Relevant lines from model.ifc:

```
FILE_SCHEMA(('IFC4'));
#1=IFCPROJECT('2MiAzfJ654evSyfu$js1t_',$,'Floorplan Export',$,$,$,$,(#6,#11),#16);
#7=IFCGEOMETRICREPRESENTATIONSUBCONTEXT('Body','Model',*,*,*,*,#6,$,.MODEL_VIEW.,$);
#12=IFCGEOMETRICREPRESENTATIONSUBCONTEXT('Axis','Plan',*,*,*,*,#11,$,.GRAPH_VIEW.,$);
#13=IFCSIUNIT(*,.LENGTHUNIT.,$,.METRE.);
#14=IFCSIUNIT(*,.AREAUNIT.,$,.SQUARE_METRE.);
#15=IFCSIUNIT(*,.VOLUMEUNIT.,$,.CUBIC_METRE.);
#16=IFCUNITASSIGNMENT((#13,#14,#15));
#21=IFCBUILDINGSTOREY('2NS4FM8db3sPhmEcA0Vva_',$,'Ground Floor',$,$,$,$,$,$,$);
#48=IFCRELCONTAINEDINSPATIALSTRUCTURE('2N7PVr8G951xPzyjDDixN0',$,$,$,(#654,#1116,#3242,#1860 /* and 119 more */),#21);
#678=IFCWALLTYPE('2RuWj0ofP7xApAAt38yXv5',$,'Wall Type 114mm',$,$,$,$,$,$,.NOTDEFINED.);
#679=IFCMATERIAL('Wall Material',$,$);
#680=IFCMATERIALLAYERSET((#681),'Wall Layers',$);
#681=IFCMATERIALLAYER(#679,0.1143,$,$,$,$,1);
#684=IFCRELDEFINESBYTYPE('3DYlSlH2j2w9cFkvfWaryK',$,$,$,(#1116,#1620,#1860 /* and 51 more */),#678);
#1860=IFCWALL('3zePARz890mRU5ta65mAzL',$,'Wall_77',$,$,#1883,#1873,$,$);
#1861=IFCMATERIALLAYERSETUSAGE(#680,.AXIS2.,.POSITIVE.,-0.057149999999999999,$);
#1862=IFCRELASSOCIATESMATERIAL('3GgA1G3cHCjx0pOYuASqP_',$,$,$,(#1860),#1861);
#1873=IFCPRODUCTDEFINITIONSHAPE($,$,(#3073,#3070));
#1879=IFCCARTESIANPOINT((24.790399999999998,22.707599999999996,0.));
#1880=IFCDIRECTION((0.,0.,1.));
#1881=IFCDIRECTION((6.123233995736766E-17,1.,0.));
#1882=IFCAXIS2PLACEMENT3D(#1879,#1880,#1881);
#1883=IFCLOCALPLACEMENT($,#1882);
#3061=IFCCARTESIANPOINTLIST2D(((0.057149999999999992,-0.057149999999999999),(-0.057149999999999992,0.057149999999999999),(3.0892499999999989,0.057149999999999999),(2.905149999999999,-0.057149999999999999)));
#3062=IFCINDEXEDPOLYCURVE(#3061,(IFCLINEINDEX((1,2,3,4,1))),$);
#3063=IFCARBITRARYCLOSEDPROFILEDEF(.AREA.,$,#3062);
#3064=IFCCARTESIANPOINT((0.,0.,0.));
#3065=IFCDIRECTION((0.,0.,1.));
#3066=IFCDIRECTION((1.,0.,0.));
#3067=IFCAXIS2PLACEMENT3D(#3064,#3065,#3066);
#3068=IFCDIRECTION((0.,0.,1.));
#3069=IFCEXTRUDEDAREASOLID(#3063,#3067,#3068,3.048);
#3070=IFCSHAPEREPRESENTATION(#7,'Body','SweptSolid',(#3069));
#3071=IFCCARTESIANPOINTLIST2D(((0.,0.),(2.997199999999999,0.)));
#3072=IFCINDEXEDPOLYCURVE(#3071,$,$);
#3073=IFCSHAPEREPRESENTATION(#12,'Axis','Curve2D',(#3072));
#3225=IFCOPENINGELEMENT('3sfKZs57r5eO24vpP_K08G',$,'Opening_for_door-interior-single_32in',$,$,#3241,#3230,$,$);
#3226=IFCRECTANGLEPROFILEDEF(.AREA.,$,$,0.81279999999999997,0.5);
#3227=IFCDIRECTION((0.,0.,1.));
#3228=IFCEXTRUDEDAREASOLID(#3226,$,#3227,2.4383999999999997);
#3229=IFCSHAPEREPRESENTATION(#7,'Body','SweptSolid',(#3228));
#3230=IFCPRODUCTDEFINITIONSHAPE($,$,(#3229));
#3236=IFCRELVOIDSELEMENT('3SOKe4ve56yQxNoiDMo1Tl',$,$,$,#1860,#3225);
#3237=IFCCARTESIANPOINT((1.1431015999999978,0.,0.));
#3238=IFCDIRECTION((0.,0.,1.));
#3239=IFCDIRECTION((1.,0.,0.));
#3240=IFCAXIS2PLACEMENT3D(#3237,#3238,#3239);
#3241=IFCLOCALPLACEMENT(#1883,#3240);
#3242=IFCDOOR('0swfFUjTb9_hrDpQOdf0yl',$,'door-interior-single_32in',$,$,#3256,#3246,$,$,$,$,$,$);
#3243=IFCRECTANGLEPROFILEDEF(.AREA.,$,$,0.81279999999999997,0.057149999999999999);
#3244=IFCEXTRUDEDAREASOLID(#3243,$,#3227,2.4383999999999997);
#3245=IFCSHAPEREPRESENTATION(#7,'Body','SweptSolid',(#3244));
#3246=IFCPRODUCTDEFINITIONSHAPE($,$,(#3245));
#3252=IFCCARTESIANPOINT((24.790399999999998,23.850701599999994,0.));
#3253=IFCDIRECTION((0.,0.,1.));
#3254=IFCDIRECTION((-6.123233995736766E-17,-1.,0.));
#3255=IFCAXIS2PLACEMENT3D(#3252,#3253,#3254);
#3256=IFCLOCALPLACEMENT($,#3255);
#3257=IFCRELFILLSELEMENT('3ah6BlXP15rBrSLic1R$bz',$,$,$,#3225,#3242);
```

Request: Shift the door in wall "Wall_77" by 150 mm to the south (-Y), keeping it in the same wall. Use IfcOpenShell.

```python
import ifcopenshell
import ifcopenshell.api.geometry
import ifcopenshell.util.placement
import ifcopenshell.util.unit

model = ifcopenshell.open("model.ifc")
unit_scale = ifcopenshell.util.unit.calculate_unit_scale(model)

door = model.by_guid("0swfFUjTb9_hrDpQOdf0yl")
opening = door.FillsVoids[0].RelatingOpeningElement
wall = opening.VoidsElements[0].RelatingBuildingElement

wall_matrix = ifcopenshell.util.placement.get_local_placement(wall.ObjectPlacement)
shift = wall_matrix[:3, 0] * -0.15 / unit_scale
before = ifcopenshell.util.placement.get_local_placement(door.ObjectPlacement)[:3, 3].copy()

# The door is not placed relative to its opening, so move both.
for product in (opening, door):
    matrix = ifcopenshell.util.placement.get_local_placement(product.ObjectPlacement)
    matrix[:3, 3] += shift
    ifcopenshell.api.geometry.edit_object_placement(model, product=product, matrix=matrix, is_si=False)

after = ifcopenshell.util.placement.get_local_placement(door.ObjectPlacement)[:3, 3]
print("door moved by", (after - before).round(3) + 0.0)

model.write("model_v2.ifc")
```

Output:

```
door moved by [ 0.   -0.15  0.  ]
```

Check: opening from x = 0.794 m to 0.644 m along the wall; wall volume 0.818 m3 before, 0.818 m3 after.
